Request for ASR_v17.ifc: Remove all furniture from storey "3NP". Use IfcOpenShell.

First a look at what the model holds.

```python
import ifcopenshell
import ifcopenshell.util.element

model = ifcopenshell.open("ASR_v17.ifc")
print(model.schema)
storey = next(s for s in model.by_type("IfcBuildingStorey") if s.Name == "3NP")
furniture = [e for e in ifcopenshell.util.element.get_decomposition(storey) if e.is_a("IfcFurnishingElement")]
seen = {}
for e in furniture:
    element_type = ifcopenshell.util.element.get_type(e)
    name = element_type.Name if element_type not in (None, e) else None
    seen[name] = seen.get(name, 0) + 1
for name, count in sorted(seen.items(), key=str):
    print(count, "x", name)
```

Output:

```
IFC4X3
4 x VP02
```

```python
import ifcopenshell
import ifcopenshell.api.root
import ifcopenshell.util.element

model = ifcopenshell.open("ASR_v17.ifc")

storey = next(s for s in model.by_type("IfcBuildingStorey") if s.Name == "3NP")
furniture = [e for e in ifcopenshell.util.element.get_decomposition(storey) if e.is_a("IfcFurnishingElement")]

for e in furniture:
    ifcopenshell.api.root.remove_product(model, product=e)
print(len(furniture), "removed")

model.write("ASR_v17_updated.ifc")
```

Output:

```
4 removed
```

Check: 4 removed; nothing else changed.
